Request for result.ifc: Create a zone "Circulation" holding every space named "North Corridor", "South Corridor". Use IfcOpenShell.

First a look at what the model holds.

```python
import ifcopenshell

model = ifcopenshell.open("result.ifc")
print(model.schema)
seen = {}
for space in model.by_type("IfcSpace"):
    seen[space.Name] = seen.get(space.Name, 0) + 1
for name, count in sorted(seen.items(), key=str):
    print(count, "x", name)
print("zones:", [z.Name for z in model.by_type("IfcZone")][:20])
```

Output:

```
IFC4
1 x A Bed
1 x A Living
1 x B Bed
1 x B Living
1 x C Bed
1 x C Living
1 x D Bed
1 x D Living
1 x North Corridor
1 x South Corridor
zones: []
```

```python
import ifcopenshell
import ifcopenshell.api.group
import ifcopenshell.api.root

model = ifcopenshell.open("result.ifc")

names = {"North Corridor", "South Corridor"}
spaces = [s for s in model.by_type("IfcSpace") if s.Name in names]

zone = ifcopenshell.api.root.create_entity(model, ifc_class="IfcZone", name="Circulation")
ifcopenshell.api.group.assign_group(model, products=spaces, group=zone)
print(len(spaces), "spaces in", zone.Name)

model.write("result_edited.ifc")
```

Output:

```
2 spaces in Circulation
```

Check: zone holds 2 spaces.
